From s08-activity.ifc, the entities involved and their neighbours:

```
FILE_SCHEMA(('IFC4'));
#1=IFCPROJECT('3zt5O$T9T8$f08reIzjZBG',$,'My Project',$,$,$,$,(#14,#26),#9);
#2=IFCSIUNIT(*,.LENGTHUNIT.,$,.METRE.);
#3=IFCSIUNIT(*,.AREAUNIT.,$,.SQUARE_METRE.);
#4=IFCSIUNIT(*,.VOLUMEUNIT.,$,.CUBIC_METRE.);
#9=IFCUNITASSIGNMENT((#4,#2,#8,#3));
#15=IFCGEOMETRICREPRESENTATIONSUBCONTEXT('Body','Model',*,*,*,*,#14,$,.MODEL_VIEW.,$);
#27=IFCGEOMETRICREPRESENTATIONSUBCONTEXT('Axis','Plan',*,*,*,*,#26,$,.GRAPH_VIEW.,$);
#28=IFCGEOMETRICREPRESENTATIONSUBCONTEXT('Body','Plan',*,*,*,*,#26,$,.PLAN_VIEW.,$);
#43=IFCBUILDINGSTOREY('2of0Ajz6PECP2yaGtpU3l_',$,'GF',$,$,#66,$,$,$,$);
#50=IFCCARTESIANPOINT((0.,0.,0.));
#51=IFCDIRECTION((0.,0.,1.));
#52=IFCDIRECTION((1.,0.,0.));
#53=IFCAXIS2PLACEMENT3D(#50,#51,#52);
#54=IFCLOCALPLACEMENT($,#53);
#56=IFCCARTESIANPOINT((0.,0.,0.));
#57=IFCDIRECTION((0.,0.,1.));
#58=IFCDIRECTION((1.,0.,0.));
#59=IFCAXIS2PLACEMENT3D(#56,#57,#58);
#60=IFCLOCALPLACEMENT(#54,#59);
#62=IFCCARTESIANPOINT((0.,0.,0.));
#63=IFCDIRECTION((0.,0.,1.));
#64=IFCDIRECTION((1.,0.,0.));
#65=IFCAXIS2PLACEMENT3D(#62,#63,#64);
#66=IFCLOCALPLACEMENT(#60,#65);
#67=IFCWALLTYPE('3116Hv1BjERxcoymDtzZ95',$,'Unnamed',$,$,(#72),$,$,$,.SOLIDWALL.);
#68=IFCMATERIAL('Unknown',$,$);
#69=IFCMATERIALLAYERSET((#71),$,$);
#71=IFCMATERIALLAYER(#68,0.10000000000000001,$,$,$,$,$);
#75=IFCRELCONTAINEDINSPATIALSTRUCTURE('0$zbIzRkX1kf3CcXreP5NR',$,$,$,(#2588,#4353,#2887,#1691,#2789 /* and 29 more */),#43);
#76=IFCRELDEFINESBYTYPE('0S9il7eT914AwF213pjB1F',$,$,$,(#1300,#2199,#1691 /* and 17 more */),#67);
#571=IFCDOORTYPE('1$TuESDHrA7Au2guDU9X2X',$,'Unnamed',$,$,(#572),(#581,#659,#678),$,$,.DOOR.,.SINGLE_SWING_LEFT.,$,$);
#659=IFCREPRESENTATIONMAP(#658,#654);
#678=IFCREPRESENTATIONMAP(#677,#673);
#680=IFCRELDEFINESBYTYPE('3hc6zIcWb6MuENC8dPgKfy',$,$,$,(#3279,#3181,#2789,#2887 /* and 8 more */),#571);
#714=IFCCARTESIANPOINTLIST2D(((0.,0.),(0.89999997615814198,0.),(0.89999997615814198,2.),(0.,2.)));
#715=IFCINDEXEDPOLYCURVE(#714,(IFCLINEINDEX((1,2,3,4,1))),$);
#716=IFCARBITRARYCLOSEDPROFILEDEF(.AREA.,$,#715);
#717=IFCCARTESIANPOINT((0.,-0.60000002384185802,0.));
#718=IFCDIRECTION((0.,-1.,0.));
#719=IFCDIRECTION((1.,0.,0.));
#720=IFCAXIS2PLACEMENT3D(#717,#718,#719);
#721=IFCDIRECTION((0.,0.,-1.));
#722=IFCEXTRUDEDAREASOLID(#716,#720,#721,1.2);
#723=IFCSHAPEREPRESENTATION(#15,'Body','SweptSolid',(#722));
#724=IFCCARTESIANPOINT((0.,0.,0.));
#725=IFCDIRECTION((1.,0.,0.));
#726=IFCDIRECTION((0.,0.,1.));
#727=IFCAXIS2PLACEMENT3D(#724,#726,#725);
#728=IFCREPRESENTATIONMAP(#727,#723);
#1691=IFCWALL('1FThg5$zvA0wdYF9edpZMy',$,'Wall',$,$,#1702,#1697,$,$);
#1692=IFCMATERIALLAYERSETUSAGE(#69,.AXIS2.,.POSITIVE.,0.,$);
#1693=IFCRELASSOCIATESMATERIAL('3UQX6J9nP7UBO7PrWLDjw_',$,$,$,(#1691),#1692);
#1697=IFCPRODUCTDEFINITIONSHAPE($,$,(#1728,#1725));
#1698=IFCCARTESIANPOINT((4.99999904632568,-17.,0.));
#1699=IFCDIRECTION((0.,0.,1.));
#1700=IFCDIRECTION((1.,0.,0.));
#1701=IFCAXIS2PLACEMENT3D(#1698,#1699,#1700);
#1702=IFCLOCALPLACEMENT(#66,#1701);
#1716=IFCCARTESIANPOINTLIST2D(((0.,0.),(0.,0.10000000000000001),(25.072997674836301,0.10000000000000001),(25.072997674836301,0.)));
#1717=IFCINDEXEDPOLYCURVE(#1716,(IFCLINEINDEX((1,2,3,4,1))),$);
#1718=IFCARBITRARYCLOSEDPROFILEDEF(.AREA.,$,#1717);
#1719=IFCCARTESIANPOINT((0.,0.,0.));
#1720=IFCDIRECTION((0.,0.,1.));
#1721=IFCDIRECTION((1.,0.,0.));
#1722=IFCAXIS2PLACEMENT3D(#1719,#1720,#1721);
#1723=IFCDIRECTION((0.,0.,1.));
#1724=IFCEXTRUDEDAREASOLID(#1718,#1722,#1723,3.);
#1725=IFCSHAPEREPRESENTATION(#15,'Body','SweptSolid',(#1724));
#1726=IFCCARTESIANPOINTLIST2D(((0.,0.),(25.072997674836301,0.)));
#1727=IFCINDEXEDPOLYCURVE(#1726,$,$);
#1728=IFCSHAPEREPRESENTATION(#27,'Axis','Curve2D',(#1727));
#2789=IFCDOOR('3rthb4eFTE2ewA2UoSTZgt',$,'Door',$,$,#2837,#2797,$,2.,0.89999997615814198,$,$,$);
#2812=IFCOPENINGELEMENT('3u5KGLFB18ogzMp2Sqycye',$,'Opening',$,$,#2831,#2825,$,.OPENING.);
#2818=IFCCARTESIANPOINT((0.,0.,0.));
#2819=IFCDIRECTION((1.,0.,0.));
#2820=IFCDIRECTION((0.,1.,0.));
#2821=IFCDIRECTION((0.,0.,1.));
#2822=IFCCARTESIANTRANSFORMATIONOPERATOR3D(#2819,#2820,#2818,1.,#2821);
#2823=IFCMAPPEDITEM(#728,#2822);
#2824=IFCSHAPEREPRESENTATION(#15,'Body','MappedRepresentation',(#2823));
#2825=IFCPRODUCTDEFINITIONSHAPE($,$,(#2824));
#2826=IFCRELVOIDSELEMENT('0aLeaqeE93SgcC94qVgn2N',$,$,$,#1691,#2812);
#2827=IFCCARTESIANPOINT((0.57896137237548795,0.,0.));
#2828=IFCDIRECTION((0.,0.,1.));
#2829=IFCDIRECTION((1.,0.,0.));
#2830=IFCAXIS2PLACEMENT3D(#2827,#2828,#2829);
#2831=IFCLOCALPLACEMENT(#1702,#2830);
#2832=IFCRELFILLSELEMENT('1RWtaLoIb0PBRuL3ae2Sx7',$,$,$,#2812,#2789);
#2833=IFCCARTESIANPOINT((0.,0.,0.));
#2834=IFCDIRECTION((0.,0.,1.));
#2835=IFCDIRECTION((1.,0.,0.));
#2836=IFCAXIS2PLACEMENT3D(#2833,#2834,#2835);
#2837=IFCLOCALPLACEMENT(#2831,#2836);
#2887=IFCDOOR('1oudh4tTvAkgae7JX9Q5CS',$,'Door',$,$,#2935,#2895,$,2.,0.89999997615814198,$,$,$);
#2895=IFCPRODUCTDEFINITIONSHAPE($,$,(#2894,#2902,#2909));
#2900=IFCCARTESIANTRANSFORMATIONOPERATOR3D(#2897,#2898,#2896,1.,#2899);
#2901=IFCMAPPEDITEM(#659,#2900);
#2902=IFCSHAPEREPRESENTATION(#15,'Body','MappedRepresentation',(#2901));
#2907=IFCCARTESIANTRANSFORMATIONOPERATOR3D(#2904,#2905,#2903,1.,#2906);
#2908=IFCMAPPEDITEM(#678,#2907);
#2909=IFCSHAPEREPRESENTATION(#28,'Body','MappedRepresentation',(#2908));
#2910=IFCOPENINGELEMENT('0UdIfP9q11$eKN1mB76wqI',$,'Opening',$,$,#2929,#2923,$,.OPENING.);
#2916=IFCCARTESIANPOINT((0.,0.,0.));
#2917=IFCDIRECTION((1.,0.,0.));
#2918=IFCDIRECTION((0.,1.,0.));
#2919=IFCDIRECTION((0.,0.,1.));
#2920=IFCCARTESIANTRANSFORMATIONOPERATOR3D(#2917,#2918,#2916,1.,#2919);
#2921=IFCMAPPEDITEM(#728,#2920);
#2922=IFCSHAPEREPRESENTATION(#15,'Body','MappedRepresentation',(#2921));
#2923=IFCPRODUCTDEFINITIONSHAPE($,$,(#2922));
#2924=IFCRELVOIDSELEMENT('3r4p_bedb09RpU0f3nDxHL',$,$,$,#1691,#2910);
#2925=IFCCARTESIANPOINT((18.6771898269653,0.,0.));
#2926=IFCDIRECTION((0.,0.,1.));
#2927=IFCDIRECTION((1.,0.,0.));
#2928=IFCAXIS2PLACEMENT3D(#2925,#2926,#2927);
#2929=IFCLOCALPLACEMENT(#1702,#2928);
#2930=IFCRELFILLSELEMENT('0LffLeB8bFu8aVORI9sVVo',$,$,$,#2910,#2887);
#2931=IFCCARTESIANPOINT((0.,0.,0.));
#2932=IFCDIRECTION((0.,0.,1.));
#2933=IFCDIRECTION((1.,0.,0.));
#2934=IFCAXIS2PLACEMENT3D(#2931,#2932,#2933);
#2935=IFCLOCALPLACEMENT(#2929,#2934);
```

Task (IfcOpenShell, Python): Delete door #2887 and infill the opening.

```python
import ifcopenshell
import ifcopenshell.api.feature
import ifcopenshell.api.root
import ifcopenshell.geom
import ifcopenshell.util.shape

model = ifcopenshell.open("s08-activity.ifc")
settings = ifcopenshell.geom.settings()


def volume(element):
    """Net volume in cubic metres, openings subtracted."""
    shape = ifcopenshell.geom.create_shape(settings, element)
    return ifcopenshell.util.shape.get_volume(shape.geometry)


door = model.by_id(2887)
opening = door.FillsVoids[0].RelatingOpeningElement
wall = opening.VoidsElements[0].RelatingBuildingElement
before = volume(wall)

ifcopenshell.api.root.remove_product(model, product=door)
ifcopenshell.api.feature.remove_feature(model, feature=opening)

after = volume(wall)

print(f"wall volume {before:.3f} -> {after:.3f} m3")

model.write("s08-activity-out.ifc")
```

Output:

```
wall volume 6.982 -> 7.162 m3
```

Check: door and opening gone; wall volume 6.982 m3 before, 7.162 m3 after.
